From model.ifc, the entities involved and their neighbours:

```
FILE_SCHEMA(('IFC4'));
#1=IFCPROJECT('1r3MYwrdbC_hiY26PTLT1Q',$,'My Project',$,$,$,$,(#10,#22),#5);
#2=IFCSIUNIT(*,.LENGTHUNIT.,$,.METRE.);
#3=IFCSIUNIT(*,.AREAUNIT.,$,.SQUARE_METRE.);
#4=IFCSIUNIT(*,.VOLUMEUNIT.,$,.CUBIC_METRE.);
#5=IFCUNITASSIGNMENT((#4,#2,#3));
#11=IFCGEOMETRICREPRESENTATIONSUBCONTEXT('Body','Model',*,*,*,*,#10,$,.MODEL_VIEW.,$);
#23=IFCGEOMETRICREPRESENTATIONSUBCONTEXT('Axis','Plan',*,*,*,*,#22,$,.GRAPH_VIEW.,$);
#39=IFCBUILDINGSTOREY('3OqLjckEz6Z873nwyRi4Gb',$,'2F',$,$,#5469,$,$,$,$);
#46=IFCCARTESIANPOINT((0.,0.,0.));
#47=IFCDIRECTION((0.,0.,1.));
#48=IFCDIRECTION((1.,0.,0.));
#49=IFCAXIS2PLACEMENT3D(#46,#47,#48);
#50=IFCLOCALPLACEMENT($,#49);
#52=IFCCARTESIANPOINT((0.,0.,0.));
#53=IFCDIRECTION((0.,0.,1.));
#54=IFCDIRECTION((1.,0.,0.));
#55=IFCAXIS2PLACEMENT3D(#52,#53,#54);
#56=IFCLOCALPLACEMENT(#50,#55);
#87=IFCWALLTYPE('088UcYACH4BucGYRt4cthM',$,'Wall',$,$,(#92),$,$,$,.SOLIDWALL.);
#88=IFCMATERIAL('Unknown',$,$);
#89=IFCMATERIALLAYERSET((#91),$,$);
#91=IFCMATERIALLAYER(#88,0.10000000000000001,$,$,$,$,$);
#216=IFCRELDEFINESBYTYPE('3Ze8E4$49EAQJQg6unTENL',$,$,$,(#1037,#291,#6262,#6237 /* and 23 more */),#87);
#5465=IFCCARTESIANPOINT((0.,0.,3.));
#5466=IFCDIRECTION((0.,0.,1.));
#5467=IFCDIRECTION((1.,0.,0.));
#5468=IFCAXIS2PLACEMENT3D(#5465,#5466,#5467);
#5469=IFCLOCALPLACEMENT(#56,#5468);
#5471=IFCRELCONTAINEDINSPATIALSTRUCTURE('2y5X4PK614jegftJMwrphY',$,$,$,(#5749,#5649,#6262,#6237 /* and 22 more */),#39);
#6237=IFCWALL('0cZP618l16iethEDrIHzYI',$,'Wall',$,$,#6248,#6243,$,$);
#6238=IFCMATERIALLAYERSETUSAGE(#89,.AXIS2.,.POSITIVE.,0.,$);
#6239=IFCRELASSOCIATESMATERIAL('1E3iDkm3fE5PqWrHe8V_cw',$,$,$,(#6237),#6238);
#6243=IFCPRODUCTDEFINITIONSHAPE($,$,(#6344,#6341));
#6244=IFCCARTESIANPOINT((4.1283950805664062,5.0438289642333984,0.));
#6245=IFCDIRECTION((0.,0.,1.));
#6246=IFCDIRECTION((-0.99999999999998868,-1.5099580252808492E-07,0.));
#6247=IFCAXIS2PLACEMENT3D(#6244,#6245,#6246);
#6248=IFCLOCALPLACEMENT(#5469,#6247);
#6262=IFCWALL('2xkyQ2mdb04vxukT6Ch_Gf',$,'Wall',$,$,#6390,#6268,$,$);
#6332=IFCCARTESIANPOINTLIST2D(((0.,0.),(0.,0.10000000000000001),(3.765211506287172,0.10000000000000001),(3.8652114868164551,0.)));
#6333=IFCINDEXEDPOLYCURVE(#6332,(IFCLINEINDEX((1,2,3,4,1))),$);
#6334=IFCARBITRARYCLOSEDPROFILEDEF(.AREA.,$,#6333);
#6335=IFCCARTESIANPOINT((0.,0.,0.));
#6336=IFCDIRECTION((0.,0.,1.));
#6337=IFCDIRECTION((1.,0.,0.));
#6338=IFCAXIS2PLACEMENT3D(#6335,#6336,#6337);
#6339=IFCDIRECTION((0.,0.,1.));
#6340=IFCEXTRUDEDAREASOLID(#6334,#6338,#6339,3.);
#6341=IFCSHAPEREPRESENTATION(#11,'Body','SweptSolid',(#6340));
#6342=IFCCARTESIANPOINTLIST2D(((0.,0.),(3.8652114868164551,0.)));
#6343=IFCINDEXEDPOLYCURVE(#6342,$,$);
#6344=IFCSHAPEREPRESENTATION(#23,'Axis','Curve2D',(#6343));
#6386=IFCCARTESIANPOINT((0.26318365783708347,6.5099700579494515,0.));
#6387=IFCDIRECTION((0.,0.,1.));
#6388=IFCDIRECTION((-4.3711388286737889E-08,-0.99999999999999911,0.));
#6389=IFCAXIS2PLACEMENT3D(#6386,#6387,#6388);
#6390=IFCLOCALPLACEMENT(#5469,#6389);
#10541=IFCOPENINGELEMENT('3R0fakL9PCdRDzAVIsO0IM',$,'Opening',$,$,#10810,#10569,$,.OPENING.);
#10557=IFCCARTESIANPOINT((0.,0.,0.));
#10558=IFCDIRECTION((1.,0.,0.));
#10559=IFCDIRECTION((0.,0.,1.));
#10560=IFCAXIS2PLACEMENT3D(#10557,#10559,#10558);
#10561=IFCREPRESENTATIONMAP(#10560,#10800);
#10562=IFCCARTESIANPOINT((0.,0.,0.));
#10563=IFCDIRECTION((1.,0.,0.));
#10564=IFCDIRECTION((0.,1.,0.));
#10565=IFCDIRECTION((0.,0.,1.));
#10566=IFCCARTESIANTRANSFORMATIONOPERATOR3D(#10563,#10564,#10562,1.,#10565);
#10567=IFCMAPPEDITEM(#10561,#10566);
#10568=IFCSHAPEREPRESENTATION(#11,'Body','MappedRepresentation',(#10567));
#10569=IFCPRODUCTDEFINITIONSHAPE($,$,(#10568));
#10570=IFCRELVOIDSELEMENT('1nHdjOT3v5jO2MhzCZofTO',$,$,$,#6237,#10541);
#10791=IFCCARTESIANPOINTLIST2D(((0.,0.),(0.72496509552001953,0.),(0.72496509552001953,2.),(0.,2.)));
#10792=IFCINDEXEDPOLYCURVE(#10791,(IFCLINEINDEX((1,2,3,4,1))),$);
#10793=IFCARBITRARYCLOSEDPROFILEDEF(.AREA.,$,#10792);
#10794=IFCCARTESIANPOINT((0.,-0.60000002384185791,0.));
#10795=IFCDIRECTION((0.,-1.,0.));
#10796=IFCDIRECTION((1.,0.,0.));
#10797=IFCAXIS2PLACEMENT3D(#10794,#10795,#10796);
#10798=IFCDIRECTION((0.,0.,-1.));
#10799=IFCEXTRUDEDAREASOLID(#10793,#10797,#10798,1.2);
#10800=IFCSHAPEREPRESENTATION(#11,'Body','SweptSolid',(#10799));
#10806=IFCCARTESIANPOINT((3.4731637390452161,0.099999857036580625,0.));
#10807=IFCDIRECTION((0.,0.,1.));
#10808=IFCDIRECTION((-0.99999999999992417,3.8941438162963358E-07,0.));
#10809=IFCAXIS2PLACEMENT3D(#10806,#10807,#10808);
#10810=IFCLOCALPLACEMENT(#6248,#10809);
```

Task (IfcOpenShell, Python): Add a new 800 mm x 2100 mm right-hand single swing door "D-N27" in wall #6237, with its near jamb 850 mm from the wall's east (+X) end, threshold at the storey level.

```python
import numpy as np
import ifcopenshell
import ifcopenshell.api.feature
import ifcopenshell.api.geometry
import ifcopenshell.api.root
import ifcopenshell.api.spatial
import ifcopenshell.geom
import ifcopenshell.util.element
import ifcopenshell.util.placement
import ifcopenshell.util.representation
import ifcopenshell.util.shape
import ifcopenshell.util.unit

model = ifcopenshell.open("model.ifc")
unit_scale = ifcopenshell.util.unit.calculate_unit_scale(model)
settings = ifcopenshell.geom.settings()


def volume(element):
    """Net volume in cubic metres, openings subtracted."""
    shape = ifcopenshell.geom.create_shape(settings, element)
    return ifcopenshell.util.shape.get_volume(shape.geometry)


wall = model.by_id(6237)
storey = ifcopenshell.util.element.get_container(wall, ifc_class="IfcBuildingStorey")
context = ifcopenshell.util.representation.get_context(model, "Model", "Body", "MODEL_VIEW")
before = volume(wall)

width, height, from_end, sill = 0.8, 2.1, 0.85, 0.0  # metres

# The wall runs along its own X axis, and the end named is its -X end.
wall_shape = ifcopenshell.geom.create_shape(settings, wall)
x, y, z = ifcopenshell.util.shape.get_vertices(wall_shape.geometry).T
start = x.min() + from_end
face, thickness = float(y.min()), float(y.max() - y.min())
wall_matrix = ifcopenshell.util.placement.get_local_placement(wall.ObjectPlacement)
level = ifcopenshell.util.placement.get_local_placement(storey.ObjectPlacement)[2, 3]


def in_wall(x, y):
    """Placement at x, y metres in the wall's axes, at sill height."""
    matrix = wall_matrix.copy()
    matrix[:, 3] = wall_matrix @ np.array([x / unit_scale, y / unit_scale, 0.0, 1.0])
    matrix[2, 3] = level + sill / unit_scale
    return matrix


# Opening: a box that overshoots both wall faces by 50 mm.
opening = ifcopenshell.api.root.create_entity(model, ifc_class="IfcOpeningElement", predefined_type="OPENING")
box = ifcopenshell.api.geometry.add_wall_representation(
    model, context=context, length=width, height=height, thickness=thickness + 0.1
)
ifcopenshell.api.geometry.assign_representation(model, product=opening, representation=box)
ifcopenshell.api.geometry.edit_object_placement(model, product=opening, matrix=in_wall(start, face - 0.05), is_si=False)
ifcopenshell.api.feature.add_feature(model, feature=opening, element=wall)

door = ifcopenshell.api.root.create_entity(model, ifc_class="IfcDoor", name="D-N27", predefined_type="DOOR")
door.OverallWidth, door.OverallHeight = width / unit_scale, height / unit_scale
door.OperationType = "SINGLE_SWING_RIGHT"
body = ifcopenshell.api.geometry.add_door_representation(
    model,
    context=context,
    overall_width=door.OverallWidth,
    overall_height=door.OverallHeight,
    operation_type="SINGLE_SWING_RIGHT",
    lining_properties={"LiningDepth": thickness / unit_scale, "ThresholdDepth": thickness / unit_scale},
)
ifcopenshell.api.geometry.assign_representation(model, product=door, representation=body)
ifcopenshell.api.spatial.assign_container(model, products=[door], relating_structure=storey)
ifcopenshell.api.feature.add_filling(model, opening=opening, element=door)

# The lining spans the wall, so the door starts at the wall face.
ifcopenshell.api.geometry.edit_object_placement(model, product=door, matrix=in_wall(start, face), is_si=False)

after = volume(wall)

print(f"wall volume {before:.3f} -> {after:.3f} m3")

model.write("model_rev.ifc")
```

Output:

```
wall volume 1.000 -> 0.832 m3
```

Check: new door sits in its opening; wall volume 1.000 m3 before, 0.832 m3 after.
